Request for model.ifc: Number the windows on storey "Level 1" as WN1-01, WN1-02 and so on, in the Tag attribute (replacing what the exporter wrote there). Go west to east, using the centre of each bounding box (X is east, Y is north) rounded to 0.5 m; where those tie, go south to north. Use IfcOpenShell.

First a look at what the model holds.

```python
import ifcopenshell
import ifcopenshell.util.element
import ifcopenshell.util.placement

model = ifcopenshell.open("model.ifc")
print(model.schema)
storey = next(s for s in model.by_type("IfcBuildingStorey") if s.Name == "Level 1")
windows = [e for e in ifcopenshell.util.element.get_decomposition(storey) if e.is_a("IfcWindow")]
for e in sorted(windows, key=lambda e: e.id()):
    origin = ifcopenshell.util.placement.get_local_placement(e.ObjectPlacement)[:3, 3]
    print(e.id(), e.Tag, e.Name, origin.round(2) + 0.0, sep=" | ")
```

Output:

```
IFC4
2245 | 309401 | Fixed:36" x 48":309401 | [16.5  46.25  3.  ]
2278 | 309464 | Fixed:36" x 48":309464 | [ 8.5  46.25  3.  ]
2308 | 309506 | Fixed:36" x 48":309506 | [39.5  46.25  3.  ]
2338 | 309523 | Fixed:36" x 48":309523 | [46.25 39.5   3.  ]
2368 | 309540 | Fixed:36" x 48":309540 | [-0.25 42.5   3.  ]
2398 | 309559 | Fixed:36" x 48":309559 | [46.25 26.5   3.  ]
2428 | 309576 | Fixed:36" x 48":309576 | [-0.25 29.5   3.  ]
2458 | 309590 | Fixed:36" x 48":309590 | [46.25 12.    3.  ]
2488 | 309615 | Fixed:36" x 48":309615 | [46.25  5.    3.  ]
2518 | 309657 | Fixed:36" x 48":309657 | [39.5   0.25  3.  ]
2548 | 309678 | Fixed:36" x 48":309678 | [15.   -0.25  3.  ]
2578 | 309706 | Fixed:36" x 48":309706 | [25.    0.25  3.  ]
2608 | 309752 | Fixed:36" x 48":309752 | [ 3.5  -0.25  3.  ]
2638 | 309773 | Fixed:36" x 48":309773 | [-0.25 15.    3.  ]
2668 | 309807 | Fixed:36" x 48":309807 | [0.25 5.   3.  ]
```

```python
import ifcopenshell
import ifcopenshell.geom
import ifcopenshell.util.element
import ifcopenshell.util.shape

model = ifcopenshell.open("model.ifc")
settings = ifcopenshell.geom.settings()
settings.set("use-world-coords", True)


def centre(element):
    shape = ifcopenshell.geom.create_shape(settings, element)
    return ifcopenshell.util.shape.get_bbox_centroid(shape.geometry)


storey = next(s for s in model.by_type("IfcBuildingStorey") if s.Name == "Level 1")
windows = [e for e in ifcopenshell.util.element.get_decomposition(storey) if e.is_a("IfcWindow")]

# Insertion points can sit at a corner or the storey origin, so sort by the geometry (in metres).
centres = {e: centre(e) for e in windows}
windows.sort(key=lambda e: (round(centres[e][0] / 0.5), centres[e][1]))

for i, e in enumerate(windows, start=1):
    number = f"WN1-{i:02d}"
    e.Tag = number
    print(e.id(), number)

model.write("model-out.ifc")
```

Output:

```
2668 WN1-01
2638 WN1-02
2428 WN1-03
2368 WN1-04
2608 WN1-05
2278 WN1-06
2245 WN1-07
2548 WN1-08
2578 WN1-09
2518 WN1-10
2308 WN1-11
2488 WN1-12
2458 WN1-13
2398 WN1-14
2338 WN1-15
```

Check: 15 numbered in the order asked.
